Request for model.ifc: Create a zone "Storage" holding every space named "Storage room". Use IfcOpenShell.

First a look at what the model holds.

```python
import ifcopenshell

model = ifcopenshell.open("model.ifc")
print(model.schema)
seen = {}
for space in model.by_type("IfcSpace"):
    seen[space.LongName] = seen.get(space.LongName, 0) + 1
for name, count in sorted(seen.items(), key=str):
    print(count, "x", name)
print("zones:", [z.Name for z in model.by_type("IfcZone")][:20])
```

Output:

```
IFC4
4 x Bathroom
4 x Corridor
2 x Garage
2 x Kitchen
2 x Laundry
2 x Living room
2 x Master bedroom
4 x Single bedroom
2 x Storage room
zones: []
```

```python
import ifcopenshell
import ifcopenshell.api.group
import ifcopenshell.api.root

model = ifcopenshell.open("model.ifc")

names = {"Storage room"}
spaces = [s for s in model.by_type("IfcSpace") if s.LongName in names]

zone = ifcopenshell.api.root.create_entity(model, ifc_class="IfcZone", name="Storage")
ifcopenshell.api.group.assign_group(model, products=spaces, group=zone)
print(len(spaces), "spaces in", zone.Name)

model.write("model_rev.ifc")
```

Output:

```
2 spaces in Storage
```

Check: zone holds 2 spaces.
